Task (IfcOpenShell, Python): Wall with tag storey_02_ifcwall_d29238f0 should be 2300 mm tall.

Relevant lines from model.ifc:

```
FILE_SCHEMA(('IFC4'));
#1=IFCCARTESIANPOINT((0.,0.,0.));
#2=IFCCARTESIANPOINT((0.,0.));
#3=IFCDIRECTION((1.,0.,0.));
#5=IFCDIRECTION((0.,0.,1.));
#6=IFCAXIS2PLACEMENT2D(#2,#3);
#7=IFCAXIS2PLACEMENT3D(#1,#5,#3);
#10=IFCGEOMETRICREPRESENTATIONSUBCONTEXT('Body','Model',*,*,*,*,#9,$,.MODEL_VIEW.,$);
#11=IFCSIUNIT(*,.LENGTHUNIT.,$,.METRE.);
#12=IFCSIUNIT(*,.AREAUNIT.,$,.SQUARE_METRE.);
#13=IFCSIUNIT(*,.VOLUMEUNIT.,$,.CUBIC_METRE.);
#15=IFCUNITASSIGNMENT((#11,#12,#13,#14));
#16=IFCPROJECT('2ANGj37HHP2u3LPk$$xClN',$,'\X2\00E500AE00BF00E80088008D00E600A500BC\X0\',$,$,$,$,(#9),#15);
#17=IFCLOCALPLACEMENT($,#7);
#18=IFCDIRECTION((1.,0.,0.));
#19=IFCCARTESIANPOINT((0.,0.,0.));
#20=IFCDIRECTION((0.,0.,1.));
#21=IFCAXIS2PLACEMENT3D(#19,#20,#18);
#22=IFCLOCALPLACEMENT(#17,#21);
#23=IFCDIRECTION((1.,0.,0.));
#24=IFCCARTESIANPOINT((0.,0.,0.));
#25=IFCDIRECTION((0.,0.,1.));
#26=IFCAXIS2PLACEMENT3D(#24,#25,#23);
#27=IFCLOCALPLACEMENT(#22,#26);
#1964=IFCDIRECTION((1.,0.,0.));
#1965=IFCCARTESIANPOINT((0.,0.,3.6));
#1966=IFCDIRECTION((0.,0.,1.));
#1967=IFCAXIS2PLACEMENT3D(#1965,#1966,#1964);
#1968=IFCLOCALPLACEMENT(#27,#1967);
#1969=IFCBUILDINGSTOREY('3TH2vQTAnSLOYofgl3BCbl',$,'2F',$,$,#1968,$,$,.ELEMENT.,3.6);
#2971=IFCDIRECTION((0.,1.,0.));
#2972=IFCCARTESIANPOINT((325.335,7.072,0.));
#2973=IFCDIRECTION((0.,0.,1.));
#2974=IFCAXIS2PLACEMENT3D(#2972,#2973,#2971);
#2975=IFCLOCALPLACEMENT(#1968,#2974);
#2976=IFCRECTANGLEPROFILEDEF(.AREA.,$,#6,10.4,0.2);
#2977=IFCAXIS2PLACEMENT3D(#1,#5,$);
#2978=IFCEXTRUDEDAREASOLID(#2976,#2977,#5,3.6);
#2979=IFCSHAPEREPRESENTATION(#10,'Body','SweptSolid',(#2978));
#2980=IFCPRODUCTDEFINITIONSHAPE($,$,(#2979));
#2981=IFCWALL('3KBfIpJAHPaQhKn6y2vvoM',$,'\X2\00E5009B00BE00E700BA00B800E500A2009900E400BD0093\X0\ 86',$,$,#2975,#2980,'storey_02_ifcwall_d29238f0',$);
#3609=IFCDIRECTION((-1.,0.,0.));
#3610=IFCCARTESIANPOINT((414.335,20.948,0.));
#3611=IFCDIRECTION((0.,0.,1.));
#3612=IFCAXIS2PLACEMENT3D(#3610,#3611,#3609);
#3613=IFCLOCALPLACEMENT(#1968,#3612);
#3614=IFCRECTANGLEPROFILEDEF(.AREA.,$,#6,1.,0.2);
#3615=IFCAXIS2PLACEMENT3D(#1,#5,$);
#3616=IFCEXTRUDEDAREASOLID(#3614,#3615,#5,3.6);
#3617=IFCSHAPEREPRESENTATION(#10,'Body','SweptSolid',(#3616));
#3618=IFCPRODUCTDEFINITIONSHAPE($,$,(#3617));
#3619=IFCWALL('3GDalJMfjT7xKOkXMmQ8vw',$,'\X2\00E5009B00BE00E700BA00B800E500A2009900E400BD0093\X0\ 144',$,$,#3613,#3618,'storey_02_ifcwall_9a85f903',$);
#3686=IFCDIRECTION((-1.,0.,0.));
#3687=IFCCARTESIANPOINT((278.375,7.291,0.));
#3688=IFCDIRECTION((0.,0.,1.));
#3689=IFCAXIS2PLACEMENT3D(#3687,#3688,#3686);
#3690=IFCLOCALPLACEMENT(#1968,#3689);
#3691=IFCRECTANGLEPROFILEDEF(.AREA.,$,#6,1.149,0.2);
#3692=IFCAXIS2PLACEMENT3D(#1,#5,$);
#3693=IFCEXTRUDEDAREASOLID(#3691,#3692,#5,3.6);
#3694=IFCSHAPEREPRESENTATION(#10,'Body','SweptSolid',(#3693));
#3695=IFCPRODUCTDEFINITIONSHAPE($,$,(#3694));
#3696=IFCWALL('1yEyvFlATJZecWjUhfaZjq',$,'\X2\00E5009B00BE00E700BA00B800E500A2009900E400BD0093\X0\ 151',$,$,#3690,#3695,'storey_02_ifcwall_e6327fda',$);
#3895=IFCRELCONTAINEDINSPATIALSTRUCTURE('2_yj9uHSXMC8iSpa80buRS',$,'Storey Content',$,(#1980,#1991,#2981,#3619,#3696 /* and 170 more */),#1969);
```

```python
import ifcopenshell
import ifcopenshell.geom
import ifcopenshell.util.representation
import ifcopenshell.util.shape

model = ifcopenshell.open("model.ifc")
settings = ifcopenshell.geom.settings()


def volume(element):
    """Net volume in cubic metres, openings subtracted."""
    shape = ifcopenshell.geom.create_shape(settings, element)
    return ifcopenshell.util.shape.get_volume(shape.geometry)


wall = model.by_guid("3KBfIpJAHPaQhKn6y2vvoM")
before = volume(wall)

body = ifcopenshell.util.representation.get_representation(wall, "Model", "Body")
solid = body.Items[0]
old_height = solid.Depth
solid.Depth = 2.3
after = volume(wall)

print(f"height {old_height:g} -> {solid.Depth:g}, volume {before:.3f} -> {after:.3f} m3")

model.write("model_rev.ifc")
```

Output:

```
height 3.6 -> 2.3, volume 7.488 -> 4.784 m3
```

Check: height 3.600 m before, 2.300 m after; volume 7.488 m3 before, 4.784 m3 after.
